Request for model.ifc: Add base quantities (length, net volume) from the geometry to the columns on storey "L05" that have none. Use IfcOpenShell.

First a look at what the model holds.

```python
import ifcopenshell
import ifcopenshell.util.element
import ifcopenshell.util.unit

model = ifcopenshell.open("model.ifc")
print(model.schema)
for unit_type in ("LENGTHUNIT", "AREAUNIT", "VOLUMEUNIT"):
    print(unit_type, ifcopenshell.util.unit.calculate_unit_scale(model, unit_type))
storey = next(s for s in model.by_type("IfcBuildingStorey") if s.Name == "L05")
columns = [e for e in ifcopenshell.util.element.get_decomposition(storey) if e.is_a("IfcColumn")]
for e in sorted(columns, key=lambda e: e.id()):
    print(e.id(), e.is_a(), e.Name, list(ifcopenshell.util.element.get_psets(e, qtos_only=True)), sep=" | ")
```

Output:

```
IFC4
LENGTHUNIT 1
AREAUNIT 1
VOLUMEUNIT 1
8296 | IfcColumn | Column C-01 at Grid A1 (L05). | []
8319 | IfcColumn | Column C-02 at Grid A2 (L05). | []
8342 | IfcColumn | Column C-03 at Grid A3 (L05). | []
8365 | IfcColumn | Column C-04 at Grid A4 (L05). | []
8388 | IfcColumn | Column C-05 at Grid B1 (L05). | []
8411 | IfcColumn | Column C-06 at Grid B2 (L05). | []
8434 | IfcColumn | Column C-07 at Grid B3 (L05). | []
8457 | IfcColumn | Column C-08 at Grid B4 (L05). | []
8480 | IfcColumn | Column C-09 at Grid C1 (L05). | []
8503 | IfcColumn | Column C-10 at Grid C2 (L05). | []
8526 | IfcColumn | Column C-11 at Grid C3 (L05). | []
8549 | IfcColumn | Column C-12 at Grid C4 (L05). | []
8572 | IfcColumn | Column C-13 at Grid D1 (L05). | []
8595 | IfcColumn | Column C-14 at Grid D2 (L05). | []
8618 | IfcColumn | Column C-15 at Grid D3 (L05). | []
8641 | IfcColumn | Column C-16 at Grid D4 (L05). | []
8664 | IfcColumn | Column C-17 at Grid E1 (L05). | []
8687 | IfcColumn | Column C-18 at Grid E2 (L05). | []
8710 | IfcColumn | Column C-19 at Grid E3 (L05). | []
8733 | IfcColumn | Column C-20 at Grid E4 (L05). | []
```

```python
import ifcopenshell
import ifcopenshell.api.pset
import ifcopenshell.geom
import ifcopenshell.util.element
import ifcopenshell.util.shape
import ifcopenshell.util.unit

model = ifcopenshell.open("model.ifc")
unit_scale = ifcopenshell.util.unit.calculate_unit_scale(model)
volume_scale = ifcopenshell.util.unit.calculate_unit_scale(model, "VOLUMEUNIT")
settings = ifcopenshell.geom.settings()

storey = next(s for s in model.by_type("IfcBuildingStorey") if s.Name == "L05")
columns = [e for e in ifcopenshell.util.element.get_decomposition(storey) if e.is_a("IfcColumn")]

for e in sorted(columns, key=lambda e: e.id()):
    if ifcopenshell.util.element.get_psets(e, qtos_only=True, should_inherit=False):
        continue
    # Geometry comes back in metres, in the element's own axes.
    shape = ifcopenshell.geom.create_shape(settings, e)
    values = {
        "Length": ifcopenshell.util.shape.get_z(shape.geometry) / unit_scale,
        "NetVolume": ifcopenshell.util.shape.get_volume(shape.geometry) / volume_scale,
    }
    qto = ifcopenshell.api.pset.add_qto(model, product=e, name="Qto_ColumnBaseQuantities")
    ifcopenshell.api.pset.edit_qto(model, qto=qto, properties=values)
    print(e.id(), {k: round(v, 3) for k, v in values.items()})

model.write("model_v2.ifc")
```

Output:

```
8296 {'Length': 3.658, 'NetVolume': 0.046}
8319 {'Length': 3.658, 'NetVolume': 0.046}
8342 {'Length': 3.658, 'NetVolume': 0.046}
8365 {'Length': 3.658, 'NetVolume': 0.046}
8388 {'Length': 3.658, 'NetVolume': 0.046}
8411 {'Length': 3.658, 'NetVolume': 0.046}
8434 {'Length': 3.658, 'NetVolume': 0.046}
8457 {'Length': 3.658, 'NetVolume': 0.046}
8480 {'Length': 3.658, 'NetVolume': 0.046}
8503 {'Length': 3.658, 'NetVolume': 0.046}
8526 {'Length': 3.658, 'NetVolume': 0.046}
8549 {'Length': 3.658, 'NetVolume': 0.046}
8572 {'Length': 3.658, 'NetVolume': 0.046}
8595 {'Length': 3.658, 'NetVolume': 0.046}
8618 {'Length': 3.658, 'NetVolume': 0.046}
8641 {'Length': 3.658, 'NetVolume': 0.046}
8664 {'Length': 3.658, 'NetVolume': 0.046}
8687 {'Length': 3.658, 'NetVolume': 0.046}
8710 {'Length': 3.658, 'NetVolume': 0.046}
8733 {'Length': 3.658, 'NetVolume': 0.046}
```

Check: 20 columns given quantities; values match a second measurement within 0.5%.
